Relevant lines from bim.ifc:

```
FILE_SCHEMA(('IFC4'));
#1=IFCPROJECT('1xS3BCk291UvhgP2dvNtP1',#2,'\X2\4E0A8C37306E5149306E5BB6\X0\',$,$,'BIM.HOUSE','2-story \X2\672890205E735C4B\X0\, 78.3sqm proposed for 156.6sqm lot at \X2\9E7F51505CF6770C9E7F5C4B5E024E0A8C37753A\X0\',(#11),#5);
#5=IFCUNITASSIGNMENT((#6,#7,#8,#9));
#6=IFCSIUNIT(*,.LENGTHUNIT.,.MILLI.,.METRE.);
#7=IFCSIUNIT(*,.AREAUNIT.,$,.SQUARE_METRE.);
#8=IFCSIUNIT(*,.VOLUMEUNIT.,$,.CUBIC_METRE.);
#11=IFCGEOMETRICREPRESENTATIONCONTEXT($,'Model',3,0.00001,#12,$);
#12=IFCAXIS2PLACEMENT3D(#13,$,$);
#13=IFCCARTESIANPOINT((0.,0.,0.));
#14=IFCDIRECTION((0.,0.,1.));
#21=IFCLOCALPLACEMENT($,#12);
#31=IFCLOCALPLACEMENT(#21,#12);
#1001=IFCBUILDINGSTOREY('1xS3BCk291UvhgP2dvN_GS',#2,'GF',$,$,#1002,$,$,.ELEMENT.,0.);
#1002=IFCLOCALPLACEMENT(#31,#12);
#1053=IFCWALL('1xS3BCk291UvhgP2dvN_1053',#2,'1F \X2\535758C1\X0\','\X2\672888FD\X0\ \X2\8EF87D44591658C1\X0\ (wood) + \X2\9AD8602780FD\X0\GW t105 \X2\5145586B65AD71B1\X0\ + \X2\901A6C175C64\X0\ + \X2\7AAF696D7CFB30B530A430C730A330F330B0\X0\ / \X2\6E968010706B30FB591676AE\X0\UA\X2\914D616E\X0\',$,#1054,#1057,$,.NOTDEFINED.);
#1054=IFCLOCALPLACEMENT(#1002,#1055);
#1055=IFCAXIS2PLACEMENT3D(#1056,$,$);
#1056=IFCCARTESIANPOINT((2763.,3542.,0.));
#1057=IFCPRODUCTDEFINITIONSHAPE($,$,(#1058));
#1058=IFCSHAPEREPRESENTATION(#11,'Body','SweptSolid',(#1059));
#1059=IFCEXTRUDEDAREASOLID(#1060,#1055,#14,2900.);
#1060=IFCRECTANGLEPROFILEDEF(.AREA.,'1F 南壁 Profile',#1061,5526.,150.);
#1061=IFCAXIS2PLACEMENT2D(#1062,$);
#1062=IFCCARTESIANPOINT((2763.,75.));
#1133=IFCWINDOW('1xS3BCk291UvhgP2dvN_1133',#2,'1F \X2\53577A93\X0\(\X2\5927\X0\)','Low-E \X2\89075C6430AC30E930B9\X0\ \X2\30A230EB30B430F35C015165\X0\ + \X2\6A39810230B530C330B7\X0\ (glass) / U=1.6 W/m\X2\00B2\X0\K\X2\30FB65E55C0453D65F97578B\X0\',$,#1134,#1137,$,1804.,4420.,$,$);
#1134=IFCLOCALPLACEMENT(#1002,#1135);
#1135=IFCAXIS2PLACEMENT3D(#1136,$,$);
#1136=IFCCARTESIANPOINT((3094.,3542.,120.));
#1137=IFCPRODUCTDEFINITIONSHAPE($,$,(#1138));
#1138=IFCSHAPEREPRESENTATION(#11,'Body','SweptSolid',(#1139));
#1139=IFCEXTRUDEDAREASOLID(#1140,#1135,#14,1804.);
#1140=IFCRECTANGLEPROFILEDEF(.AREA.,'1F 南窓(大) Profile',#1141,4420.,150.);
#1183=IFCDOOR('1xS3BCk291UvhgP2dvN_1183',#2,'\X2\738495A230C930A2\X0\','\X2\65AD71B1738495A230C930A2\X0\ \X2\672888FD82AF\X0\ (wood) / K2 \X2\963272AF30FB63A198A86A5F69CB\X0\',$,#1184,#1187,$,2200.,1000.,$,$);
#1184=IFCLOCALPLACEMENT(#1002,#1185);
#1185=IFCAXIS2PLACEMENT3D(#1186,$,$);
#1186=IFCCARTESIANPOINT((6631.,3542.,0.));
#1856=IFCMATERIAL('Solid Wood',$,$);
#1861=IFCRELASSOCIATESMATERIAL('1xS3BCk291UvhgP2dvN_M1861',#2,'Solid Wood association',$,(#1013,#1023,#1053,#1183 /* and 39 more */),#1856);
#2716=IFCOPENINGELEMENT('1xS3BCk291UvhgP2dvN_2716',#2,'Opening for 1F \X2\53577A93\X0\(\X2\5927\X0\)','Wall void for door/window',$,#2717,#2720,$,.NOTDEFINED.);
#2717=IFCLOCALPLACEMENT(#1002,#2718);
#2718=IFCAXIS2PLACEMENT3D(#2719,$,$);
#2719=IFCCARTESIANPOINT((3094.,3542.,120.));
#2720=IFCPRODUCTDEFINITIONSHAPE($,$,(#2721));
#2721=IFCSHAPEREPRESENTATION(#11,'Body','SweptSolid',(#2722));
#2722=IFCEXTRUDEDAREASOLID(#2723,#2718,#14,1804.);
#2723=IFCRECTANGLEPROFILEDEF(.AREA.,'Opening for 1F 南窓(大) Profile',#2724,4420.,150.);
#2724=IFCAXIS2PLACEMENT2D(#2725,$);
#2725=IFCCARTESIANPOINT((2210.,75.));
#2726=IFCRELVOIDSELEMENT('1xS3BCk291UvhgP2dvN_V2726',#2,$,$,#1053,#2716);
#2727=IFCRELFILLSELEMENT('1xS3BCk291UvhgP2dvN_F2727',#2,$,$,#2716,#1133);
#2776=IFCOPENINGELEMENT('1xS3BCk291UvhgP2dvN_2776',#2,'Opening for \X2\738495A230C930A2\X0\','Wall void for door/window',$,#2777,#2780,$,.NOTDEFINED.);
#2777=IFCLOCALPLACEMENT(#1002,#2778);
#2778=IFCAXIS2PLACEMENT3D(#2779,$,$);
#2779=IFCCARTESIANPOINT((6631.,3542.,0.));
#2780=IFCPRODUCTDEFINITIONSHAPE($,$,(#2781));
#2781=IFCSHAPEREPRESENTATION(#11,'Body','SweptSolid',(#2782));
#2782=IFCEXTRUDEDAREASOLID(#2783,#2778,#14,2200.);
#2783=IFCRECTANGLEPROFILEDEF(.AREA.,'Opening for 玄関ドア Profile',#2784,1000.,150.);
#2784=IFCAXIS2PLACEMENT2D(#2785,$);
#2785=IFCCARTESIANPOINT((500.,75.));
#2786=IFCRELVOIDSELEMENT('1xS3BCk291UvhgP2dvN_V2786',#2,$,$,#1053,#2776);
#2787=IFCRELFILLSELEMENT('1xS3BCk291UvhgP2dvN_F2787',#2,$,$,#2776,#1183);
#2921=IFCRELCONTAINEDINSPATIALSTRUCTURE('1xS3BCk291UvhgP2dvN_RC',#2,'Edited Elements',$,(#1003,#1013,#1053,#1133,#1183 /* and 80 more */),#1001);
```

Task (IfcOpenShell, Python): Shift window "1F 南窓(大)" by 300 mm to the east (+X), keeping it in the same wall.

```python
import ifcopenshell
import ifcopenshell.api.geometry
import ifcopenshell.util.placement
import ifcopenshell.util.unit

model = ifcopenshell.open("bim.ifc")
unit_scale = ifcopenshell.util.unit.calculate_unit_scale(model)

window = model.by_guid("1xS3BCk291UvhgP2dvN_1133")
opening = window.FillsVoids[0].RelatingOpeningElement
wall = opening.VoidsElements[0].RelatingBuildingElement

wall_matrix = ifcopenshell.util.placement.get_local_placement(wall.ObjectPlacement)
shift = wall_matrix[:3, 0] * 0.3 / unit_scale
before = ifcopenshell.util.placement.get_local_placement(window.ObjectPlacement)[:3, 3].copy()

# The window is not placed relative to its opening, so move both.
for product in (opening, window):
    matrix = ifcopenshell.util.placement.get_local_placement(product.ObjectPlacement)
    matrix[:3, 3] += shift
    ifcopenshell.api.geometry.edit_object_placement(model, product=product, matrix=matrix, is_si=False)

after = ifcopenshell.util.placement.get_local_placement(window.ObjectPlacement)[:3, 3]
print("window moved by", (after - before).round(3) + 0.0)

model.write("bim_v2.ifc")
```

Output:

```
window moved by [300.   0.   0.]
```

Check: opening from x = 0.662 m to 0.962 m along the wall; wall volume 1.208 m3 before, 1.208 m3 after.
